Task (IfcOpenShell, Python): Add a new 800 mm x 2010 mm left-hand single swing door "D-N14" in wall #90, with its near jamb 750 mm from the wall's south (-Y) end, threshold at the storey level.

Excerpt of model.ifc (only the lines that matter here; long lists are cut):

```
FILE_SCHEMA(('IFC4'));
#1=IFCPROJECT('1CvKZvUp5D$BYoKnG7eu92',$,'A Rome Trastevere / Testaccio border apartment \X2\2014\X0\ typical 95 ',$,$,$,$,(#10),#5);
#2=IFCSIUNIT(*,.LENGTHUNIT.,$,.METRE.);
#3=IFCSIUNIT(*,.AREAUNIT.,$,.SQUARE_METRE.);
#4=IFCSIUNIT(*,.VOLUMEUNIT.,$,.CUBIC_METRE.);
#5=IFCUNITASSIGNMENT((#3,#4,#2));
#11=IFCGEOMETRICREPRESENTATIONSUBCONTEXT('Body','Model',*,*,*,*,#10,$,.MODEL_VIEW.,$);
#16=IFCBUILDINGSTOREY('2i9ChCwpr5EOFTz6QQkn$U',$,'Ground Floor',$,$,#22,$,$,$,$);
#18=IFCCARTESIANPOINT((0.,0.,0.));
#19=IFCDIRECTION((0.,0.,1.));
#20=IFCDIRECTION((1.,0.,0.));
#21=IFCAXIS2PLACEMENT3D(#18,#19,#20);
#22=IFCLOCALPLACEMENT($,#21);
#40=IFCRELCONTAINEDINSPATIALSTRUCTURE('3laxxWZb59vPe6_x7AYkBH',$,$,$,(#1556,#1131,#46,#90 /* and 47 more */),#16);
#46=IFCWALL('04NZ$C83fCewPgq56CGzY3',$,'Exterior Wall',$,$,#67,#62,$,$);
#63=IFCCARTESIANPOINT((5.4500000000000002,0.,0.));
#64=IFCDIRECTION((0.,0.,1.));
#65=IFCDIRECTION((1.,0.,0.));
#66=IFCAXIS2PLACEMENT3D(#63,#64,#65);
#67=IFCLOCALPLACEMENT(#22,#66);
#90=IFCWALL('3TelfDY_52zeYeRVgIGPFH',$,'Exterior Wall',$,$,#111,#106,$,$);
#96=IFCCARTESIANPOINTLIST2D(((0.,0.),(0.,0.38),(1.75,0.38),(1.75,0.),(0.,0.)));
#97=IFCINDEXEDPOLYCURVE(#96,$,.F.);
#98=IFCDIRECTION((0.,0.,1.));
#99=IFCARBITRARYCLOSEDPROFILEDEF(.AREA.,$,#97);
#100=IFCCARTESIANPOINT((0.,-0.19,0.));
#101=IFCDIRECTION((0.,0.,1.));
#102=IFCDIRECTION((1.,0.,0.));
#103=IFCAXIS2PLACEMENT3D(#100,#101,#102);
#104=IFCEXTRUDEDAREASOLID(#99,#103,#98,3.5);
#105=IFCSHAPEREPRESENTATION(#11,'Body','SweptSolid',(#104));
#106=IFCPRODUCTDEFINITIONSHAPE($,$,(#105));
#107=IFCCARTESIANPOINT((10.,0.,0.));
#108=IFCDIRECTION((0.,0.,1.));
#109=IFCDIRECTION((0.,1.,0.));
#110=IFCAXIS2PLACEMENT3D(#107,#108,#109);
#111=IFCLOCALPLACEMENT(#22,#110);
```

```python
import numpy as np
import ifcopenshell
import ifcopenshell.api.feature
import ifcopenshell.api.geometry
import ifcopenshell.api.root
import ifcopenshell.api.spatial
import ifcopenshell.geom
import ifcopenshell.util.element
import ifcopenshell.util.placement
import ifcopenshell.util.representation
import ifcopenshell.util.shape
import ifcopenshell.util.unit

model = ifcopenshell.open("model.ifc")
unit_scale = ifcopenshell.util.unit.calculate_unit_scale(model)
settings = ifcopenshell.geom.settings()


def volume(element):
    """Net volume in cubic metres, openings subtracted."""
    shape = ifcopenshell.geom.create_shape(settings, element)
    return ifcopenshell.util.shape.get_volume(shape.geometry)


wall = model.by_guid("3TelfDY_52zeYeRVgIGPFH")
storey = ifcopenshell.util.element.get_container(wall, ifc_class="IfcBuildingStorey")
context = ifcopenshell.util.representation.get_context(model, "Model", "Body", "MODEL_VIEW")
before = volume(wall)

width, height, from_end, sill = 0.8, 2.01, 0.75, 0.0  # metres

# The wall runs along its own X axis, and the end named is its -X end.
wall_shape = ifcopenshell.geom.create_shape(settings, wall)
x, y, z = ifcopenshell.util.shape.get_vertices(wall_shape.geometry).T
start = x.min() + from_end
face, thickness = float(y.min()), float(y.max() - y.min())
wall_matrix = ifcopenshell.util.placement.get_local_placement(wall.ObjectPlacement)
level = ifcopenshell.util.placement.get_local_placement(storey.ObjectPlacement)[2, 3]


def in_wall(x, y):
    """Placement at x, y metres in the wall's axes, at sill height."""
    matrix = wall_matrix.copy()
    matrix[:, 3] = wall_matrix @ np.array([x / unit_scale, y / unit_scale, 0.0, 1.0])
    matrix[2, 3] = level + sill / unit_scale
    return matrix


# Opening: a box that overshoots both wall faces by 50 mm.
opening = ifcopenshell.api.root.create_entity(model, ifc_class="IfcOpeningElement", predefined_type="OPENING")
box = ifcopenshell.api.geometry.add_wall_representation(
    model, context=context, length=width, height=height, thickness=thickness + 0.1
)
ifcopenshell.api.geometry.assign_representation(model, product=opening, representation=box)
ifcopenshell.api.geometry.edit_object_placement(model, product=opening, matrix=in_wall(start, face - 0.05), is_si=False)
ifcopenshell.api.feature.add_feature(model, feature=opening, element=wall)

door = ifcopenshell.api.root.create_entity(model, ifc_class="IfcDoor", name="D-N14", predefined_type="DOOR")
door.OverallWidth, door.OverallHeight = width / unit_scale, height / unit_scale
door.OperationType = "SINGLE_SWING_LEFT"
body = ifcopenshell.api.geometry.add_door_representation(
    model,
    context=context,
    overall_width=door.OverallWidth,
    overall_height=door.OverallHeight,
    operation_type="SINGLE_SWING_LEFT",
    lining_properties={"LiningDepth": thickness / unit_scale, "ThresholdDepth": thickness / unit_scale},
)
ifcopenshell.api.geometry.assign_representation(model, product=door, representation=body)
ifcopenshell.api.spatial.assign_container(model, products=[door], relating_structure=storey)
ifcopenshell.api.feature.add_filling(model, opening=opening, element=door)

# The lining spans the wall, so the door starts at the wall face.
ifcopenshell.api.geometry.edit_object_placement(model, product=door, matrix=in_wall(start, face), is_si=False)

after = volume(wall)

print(f"wall volume {before:.3f} -> {after:.3f} m3")

model.write("model_updated.ifc")
```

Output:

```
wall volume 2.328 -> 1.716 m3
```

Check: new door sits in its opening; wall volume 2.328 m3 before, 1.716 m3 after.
